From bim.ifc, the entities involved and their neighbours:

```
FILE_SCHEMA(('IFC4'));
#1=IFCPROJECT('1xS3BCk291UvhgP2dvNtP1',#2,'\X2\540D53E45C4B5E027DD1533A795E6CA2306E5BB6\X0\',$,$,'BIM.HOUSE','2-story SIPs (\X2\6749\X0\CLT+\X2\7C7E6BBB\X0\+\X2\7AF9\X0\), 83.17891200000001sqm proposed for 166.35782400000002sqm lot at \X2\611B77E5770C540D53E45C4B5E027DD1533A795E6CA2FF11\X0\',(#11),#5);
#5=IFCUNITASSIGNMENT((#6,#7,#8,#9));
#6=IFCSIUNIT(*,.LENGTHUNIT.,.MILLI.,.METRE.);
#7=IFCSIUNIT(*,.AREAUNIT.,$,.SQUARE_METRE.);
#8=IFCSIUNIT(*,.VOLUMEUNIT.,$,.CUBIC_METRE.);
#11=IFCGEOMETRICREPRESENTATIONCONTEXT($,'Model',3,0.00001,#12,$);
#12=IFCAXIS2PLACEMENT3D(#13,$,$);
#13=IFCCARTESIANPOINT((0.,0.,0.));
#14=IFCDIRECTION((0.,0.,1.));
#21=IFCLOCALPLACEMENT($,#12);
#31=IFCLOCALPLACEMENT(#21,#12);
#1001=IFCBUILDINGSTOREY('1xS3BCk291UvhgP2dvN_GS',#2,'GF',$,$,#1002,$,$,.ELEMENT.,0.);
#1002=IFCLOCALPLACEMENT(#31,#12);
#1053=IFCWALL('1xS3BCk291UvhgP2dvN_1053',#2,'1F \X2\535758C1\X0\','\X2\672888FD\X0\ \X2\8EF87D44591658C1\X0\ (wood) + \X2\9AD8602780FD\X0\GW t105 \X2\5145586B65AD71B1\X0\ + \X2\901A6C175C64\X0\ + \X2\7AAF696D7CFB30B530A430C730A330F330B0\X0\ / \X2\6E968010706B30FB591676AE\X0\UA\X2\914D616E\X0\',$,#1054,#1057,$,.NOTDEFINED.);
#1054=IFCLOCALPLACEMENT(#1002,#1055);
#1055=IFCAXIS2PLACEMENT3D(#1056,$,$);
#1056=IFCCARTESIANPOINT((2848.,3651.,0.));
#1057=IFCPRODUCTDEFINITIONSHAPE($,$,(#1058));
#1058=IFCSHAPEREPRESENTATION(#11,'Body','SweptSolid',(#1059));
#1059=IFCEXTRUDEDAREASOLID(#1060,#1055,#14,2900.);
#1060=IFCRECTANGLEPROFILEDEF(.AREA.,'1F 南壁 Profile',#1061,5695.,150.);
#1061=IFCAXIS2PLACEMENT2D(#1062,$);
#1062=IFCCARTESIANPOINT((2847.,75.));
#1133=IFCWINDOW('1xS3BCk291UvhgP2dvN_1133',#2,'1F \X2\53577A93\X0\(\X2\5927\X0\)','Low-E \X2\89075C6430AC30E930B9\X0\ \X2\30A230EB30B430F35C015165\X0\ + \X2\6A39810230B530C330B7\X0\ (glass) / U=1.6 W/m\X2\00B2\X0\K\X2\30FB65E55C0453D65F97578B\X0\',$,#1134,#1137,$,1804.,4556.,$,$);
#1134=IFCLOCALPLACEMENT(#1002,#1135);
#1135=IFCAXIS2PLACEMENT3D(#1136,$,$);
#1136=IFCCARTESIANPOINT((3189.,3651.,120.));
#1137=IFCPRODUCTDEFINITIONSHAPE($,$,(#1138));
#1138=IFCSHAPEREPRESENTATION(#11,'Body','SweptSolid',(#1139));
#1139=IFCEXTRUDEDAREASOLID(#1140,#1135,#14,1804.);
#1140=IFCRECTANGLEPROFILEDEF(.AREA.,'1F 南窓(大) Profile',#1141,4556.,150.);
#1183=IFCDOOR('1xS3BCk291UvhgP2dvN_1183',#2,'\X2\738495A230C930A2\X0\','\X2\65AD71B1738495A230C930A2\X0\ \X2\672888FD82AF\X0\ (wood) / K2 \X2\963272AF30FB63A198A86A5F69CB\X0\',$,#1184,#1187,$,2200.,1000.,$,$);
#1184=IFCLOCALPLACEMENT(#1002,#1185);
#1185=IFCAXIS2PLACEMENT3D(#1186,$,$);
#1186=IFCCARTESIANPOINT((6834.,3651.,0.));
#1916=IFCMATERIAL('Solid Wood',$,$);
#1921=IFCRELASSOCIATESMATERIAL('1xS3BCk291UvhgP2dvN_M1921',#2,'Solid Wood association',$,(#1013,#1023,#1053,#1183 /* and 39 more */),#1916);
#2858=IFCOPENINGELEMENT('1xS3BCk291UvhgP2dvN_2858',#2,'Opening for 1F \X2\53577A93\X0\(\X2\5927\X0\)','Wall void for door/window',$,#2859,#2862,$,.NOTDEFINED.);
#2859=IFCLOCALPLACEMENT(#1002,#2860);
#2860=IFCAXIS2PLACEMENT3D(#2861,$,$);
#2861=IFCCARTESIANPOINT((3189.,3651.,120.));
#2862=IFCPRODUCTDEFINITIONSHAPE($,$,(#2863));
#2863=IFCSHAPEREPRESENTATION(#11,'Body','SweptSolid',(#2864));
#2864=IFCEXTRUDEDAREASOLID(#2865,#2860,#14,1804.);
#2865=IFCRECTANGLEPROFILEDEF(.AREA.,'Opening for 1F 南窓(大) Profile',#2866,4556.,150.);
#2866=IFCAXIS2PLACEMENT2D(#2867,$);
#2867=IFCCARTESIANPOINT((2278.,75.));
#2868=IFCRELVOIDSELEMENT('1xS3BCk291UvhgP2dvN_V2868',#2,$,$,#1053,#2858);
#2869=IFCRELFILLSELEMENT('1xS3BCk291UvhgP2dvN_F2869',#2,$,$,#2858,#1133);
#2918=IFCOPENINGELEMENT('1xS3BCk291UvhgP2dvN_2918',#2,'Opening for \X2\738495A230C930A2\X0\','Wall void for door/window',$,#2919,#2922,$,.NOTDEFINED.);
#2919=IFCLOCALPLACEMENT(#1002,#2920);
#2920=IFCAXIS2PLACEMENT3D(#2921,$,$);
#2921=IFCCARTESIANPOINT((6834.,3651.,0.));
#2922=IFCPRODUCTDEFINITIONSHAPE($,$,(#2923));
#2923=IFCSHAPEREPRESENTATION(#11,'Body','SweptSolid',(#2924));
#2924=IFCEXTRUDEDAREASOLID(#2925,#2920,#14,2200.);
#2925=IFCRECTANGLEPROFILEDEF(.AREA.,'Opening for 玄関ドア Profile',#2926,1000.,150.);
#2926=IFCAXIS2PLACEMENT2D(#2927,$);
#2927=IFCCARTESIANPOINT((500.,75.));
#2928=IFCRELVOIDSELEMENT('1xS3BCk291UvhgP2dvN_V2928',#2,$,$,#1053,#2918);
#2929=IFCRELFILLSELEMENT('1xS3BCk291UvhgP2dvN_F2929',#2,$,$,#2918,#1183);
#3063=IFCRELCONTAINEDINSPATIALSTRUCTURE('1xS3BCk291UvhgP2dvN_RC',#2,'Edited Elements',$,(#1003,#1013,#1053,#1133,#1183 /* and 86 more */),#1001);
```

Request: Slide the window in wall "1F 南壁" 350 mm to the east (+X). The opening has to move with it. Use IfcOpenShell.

```python
import ifcopenshell
import ifcopenshell.api.geometry
import ifcopenshell.util.placement

model = ifcopenshell.open("bim.ifc")

window = model.by_guid("1xS3BCk291UvhgP2dvN_1133")
opening = window.FillsVoids[0].RelatingOpeningElement
wall = opening.VoidsElements[0].RelatingBuildingElement

wall_matrix = ifcopenshell.util.placement.get_local_placement(wall.ObjectPlacement)
shift = wall_matrix[:3, 0] * 350.0
before = ifcopenshell.util.placement.get_local_placement(window.ObjectPlacement)[:3, 3].copy()

# The window is not placed relative to its opening, so move both.
for product in (opening, window):
    matrix = ifcopenshell.util.placement.get_local_placement(product.ObjectPlacement)
    matrix[:3, 3] += shift
    ifcopenshell.api.geometry.edit_object_placement(model, product=product, matrix=matrix, is_si=False)

after = ifcopenshell.util.placement.get_local_placement(window.ObjectPlacement)[:3, 3]
print("window moved by", (after - before).round(3) + 0.0)

model.write("bim_rev.ifc")
```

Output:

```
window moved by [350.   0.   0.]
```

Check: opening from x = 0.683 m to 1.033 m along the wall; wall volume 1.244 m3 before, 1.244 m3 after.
